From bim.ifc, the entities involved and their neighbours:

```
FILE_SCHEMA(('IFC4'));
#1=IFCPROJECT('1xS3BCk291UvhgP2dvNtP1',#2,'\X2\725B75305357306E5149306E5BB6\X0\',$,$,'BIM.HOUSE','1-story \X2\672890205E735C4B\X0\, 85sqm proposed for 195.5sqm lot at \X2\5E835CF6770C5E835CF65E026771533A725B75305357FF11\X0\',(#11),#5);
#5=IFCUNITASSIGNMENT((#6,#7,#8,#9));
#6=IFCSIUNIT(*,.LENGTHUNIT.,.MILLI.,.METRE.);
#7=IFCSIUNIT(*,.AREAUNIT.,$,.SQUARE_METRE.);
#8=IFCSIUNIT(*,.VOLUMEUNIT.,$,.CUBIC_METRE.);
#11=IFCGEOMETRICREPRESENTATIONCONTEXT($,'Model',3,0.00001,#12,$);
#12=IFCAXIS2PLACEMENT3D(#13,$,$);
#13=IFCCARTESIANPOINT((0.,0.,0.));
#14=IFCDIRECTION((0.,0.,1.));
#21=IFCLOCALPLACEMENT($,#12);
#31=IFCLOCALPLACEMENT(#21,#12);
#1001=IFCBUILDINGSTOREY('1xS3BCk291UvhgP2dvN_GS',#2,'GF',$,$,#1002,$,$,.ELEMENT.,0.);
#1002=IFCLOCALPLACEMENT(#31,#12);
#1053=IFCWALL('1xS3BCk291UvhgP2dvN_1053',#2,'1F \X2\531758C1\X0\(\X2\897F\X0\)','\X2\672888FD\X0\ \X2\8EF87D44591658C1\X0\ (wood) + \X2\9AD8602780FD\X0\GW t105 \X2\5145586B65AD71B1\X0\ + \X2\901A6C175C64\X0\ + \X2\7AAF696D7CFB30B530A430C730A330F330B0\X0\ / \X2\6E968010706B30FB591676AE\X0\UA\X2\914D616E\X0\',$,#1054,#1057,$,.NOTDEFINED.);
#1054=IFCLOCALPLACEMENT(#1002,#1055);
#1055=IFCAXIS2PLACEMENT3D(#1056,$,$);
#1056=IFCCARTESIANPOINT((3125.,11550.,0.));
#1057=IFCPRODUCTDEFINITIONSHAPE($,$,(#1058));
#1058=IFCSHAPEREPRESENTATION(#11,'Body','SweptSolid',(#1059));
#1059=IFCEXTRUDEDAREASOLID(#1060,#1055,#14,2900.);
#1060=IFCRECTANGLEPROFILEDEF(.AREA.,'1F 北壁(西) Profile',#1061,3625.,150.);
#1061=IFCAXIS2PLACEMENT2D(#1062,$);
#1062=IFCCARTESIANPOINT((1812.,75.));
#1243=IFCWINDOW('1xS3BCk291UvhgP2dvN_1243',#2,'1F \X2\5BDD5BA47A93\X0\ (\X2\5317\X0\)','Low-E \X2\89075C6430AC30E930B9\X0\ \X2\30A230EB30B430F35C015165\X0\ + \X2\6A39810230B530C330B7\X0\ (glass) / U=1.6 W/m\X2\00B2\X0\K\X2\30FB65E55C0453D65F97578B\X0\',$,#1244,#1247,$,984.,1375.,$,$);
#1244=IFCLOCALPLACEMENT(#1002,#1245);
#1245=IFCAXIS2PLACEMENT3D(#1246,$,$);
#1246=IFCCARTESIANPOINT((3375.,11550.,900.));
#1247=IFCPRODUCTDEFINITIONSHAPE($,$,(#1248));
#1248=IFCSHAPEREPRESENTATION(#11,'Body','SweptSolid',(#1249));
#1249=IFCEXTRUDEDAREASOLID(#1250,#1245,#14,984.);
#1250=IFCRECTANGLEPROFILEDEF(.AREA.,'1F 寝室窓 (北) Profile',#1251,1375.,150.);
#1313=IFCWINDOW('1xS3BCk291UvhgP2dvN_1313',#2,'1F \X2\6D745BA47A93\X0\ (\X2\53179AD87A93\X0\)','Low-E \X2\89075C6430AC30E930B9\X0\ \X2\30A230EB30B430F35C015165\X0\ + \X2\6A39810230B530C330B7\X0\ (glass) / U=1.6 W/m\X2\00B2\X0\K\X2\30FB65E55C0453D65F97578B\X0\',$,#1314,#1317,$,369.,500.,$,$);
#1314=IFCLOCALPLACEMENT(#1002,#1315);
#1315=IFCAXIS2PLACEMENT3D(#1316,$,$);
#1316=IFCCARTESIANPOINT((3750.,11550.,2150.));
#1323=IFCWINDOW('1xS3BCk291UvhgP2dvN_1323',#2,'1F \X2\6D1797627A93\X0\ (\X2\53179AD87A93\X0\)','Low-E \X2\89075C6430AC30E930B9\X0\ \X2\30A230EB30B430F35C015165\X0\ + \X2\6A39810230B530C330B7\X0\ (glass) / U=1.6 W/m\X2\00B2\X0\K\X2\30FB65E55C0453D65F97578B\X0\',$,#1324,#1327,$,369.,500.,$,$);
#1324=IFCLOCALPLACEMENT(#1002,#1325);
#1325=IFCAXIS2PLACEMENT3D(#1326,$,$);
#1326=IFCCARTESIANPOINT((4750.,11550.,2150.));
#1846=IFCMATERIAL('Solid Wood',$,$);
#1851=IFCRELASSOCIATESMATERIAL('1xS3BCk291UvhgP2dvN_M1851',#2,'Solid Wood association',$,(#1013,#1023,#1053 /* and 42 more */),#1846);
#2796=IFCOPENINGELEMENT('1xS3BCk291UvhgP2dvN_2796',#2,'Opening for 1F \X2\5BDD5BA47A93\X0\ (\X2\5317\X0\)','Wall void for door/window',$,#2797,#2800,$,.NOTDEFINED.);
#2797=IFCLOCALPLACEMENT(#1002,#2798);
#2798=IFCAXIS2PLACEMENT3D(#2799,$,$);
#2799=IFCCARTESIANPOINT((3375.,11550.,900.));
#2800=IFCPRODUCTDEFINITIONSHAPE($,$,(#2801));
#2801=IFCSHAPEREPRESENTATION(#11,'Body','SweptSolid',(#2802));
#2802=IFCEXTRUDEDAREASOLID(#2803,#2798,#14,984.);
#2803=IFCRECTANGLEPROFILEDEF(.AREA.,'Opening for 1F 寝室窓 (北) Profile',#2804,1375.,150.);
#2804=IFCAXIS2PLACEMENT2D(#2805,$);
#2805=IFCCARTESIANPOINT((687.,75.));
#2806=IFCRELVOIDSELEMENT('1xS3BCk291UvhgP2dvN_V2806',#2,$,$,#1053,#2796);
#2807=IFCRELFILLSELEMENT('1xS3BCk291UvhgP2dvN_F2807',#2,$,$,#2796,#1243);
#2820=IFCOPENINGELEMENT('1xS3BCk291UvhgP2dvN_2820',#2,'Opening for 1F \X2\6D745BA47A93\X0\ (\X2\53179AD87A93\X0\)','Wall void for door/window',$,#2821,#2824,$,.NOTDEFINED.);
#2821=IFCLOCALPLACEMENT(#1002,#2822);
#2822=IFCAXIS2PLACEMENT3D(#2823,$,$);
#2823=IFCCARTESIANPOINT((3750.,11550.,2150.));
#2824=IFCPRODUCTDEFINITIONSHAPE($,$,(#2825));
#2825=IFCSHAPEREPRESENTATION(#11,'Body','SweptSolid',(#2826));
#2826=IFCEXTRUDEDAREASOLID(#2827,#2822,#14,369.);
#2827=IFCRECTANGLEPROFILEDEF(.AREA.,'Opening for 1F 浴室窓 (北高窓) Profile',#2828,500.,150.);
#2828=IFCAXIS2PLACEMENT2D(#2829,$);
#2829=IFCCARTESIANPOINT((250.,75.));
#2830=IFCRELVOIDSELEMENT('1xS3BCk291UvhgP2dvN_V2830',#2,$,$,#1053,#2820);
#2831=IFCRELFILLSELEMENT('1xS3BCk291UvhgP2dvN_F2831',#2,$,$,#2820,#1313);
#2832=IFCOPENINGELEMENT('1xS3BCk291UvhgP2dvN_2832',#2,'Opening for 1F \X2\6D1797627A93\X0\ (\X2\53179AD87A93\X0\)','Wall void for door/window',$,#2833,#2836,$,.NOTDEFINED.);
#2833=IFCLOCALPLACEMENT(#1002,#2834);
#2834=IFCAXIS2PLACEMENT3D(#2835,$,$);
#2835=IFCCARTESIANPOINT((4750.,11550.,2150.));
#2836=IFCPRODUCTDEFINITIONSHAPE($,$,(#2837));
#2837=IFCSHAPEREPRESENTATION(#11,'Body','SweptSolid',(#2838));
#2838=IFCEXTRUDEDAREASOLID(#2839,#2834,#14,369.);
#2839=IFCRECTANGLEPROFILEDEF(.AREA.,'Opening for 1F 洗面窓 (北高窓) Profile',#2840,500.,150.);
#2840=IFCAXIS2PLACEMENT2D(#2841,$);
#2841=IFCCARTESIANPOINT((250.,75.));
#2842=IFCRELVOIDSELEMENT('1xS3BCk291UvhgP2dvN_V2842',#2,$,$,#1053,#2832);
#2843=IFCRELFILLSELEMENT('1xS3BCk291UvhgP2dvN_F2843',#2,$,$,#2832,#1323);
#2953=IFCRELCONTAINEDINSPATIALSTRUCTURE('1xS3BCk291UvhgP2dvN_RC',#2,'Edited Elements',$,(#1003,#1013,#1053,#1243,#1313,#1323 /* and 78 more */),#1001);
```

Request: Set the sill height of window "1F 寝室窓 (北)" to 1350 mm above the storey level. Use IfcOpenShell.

```python
import numpy as np
import ifcopenshell
import ifcopenshell.api.geometry
import ifcopenshell.geom
import ifcopenshell.util.element
import ifcopenshell.util.placement
import ifcopenshell.util.shape
import ifcopenshell.util.unit

model = ifcopenshell.open("bim.ifc")
unit_scale = ifcopenshell.util.unit.calculate_unit_scale(model)

window = model.by_guid("1xS3BCk291UvhgP2dvN_1243")
opening = window.FillsVoids[0].RelatingOpeningElement
storey = ifcopenshell.util.element.get_container(window, ifc_class="IfcBuildingStorey")
level = ifcopenshell.util.placement.get_local_placement(storey.ObjectPlacement)[2, 3]

# The opening's origin need not be at the sill, so measure its lowest point.
shape = ifcopenshell.geom.create_shape(ifcopenshell.geom.settings(), opening)
bottom = ifcopenshell.util.shape.get_shape_bottom_elevation(shape, shape.geometry) / unit_scale
dz = level + 1350.0 - bottom

shift = np.array([0.0, 0.0, dz])
# The window is not placed relative to its opening, so move both.
for product in (opening, window):
    matrix = ifcopenshell.util.placement.get_local_placement(product.ObjectPlacement)
    matrix[:3, 3] += shift
    ifcopenshell.api.geometry.edit_object_placement(model, product=product, matrix=matrix, is_si=False)

print(f"moved by {dz * unit_scale:+.3f} m")

model.write("bim_rev.ifc")
```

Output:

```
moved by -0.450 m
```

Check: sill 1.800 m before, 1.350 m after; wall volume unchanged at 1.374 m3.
